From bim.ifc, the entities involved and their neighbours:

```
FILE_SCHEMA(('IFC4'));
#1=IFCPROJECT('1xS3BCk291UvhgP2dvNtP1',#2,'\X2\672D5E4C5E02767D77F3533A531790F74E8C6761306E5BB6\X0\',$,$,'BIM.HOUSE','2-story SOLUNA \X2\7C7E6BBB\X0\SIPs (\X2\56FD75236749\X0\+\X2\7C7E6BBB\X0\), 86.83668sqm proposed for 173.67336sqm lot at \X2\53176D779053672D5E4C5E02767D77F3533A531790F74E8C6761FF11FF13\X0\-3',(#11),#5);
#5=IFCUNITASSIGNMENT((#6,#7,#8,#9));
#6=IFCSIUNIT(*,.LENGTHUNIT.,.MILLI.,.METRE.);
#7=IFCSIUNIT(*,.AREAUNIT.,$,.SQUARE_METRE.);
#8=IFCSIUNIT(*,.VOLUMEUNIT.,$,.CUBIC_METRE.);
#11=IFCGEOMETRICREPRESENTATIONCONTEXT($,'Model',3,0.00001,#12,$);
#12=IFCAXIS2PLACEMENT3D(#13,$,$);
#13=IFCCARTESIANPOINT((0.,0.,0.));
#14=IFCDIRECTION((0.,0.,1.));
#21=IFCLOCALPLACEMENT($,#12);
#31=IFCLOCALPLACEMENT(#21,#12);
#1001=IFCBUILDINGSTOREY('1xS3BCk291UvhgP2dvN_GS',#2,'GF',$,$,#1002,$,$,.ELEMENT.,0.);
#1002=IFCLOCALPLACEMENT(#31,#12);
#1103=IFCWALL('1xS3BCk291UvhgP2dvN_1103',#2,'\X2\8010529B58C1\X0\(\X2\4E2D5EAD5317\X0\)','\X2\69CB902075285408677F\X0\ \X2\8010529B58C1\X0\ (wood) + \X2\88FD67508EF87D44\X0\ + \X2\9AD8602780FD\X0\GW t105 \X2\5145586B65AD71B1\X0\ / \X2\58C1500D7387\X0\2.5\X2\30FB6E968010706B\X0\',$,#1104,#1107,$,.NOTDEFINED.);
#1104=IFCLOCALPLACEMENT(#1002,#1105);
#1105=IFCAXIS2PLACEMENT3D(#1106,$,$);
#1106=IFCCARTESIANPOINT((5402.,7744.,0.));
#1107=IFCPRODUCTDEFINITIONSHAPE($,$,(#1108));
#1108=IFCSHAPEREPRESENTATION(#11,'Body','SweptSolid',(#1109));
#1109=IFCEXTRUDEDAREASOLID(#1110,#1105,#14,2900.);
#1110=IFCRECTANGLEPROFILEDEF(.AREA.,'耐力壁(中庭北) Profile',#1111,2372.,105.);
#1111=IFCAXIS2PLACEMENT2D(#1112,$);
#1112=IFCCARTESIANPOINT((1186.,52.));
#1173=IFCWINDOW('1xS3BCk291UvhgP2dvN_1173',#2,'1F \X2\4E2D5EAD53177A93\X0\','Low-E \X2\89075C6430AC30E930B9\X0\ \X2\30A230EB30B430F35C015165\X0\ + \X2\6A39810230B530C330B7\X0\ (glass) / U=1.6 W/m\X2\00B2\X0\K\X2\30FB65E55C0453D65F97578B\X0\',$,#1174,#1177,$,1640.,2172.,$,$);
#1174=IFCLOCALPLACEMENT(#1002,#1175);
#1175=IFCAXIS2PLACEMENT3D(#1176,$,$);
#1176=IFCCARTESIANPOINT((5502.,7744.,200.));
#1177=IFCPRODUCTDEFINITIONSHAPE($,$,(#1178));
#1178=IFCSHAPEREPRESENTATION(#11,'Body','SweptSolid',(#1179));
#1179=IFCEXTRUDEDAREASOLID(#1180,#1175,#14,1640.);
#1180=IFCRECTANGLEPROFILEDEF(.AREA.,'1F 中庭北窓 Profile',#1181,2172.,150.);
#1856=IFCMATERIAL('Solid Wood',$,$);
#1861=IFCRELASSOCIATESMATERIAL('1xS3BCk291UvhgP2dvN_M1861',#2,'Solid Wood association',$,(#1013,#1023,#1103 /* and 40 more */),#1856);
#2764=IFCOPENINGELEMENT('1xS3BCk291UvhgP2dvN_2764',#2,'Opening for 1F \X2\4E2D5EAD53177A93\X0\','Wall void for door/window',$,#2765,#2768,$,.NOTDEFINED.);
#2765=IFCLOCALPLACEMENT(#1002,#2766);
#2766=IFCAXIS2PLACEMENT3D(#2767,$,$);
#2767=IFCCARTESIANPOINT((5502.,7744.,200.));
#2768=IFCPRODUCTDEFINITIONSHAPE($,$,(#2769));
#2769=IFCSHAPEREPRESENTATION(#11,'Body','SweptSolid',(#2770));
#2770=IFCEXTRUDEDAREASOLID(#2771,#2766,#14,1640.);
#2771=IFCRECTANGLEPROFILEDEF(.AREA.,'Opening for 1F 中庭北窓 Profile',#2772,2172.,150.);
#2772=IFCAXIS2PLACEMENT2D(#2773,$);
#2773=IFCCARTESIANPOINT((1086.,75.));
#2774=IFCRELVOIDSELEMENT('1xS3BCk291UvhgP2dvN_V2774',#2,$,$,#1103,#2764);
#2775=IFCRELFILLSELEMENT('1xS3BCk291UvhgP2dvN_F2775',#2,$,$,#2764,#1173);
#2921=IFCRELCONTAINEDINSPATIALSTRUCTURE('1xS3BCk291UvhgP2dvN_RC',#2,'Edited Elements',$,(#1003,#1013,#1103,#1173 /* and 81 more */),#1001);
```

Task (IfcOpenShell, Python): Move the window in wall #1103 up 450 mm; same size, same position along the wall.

```python
import numpy as np
import ifcopenshell
import ifcopenshell.api.geometry
import ifcopenshell.util.placement
import ifcopenshell.util.unit

model = ifcopenshell.open("bim.ifc")
unit_scale = ifcopenshell.util.unit.calculate_unit_scale(model)

window = model.by_guid("1xS3BCk291UvhgP2dvN_1173")
opening = window.FillsVoids[0].RelatingOpeningElement
dz = 450.0

shift = np.array([0.0, 0.0, dz])
# The window is not placed relative to its opening, so move both.
for product in (opening, window):
    matrix = ifcopenshell.util.placement.get_local_placement(product.ObjectPlacement)
    matrix[:3, 3] += shift
    ifcopenshell.api.geometry.edit_object_placement(model, product=product, matrix=matrix, is_si=False)

print(f"moved by {dz * unit_scale:+.3f} m")

model.write("bim_edited.ifc")
```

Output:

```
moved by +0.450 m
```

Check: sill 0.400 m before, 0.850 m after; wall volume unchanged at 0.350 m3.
